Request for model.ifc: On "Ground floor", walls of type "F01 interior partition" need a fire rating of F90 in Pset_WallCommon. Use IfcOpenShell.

First a look at what the model holds.

```python
import ifcopenshell
import ifcopenshell.util.element

model = ifcopenshell.open("model.ifc")
print(model.schema)
storey = next(s for s in model.by_type("IfcBuildingStorey") if s.Name == "Ground floor")
walls = [e for e in ifcopenshell.util.element.get_decomposition(storey) if e.is_a("IfcWall")]
seen = {}
for e in walls:
    element_type = ifcopenshell.util.element.get_type(e)
    key = (element_type.Name if element_type != e and element_type else None, ifcopenshell.util.element.get_pset(e, "Pset_WallCommon", "FireRating"))
    seen[key] = seen.get(key, 0) + 1
for (name, value), count in sorted(seen.items(), key=str):
    print(count, "x", name, "|", value)
```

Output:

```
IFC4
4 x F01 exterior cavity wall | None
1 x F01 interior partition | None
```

```python
import ifcopenshell
import ifcopenshell.api.pset
import ifcopenshell.util.element

model = ifcopenshell.open("model.ifc")

storey = next(s for s in model.by_type("IfcBuildingStorey") if s.Name == "Ground floor")
walls = [e for e in ifcopenshell.util.element.get_decomposition(storey) if e.is_a("IfcWall")]

count = 0
for e in walls:
    element_type = ifcopenshell.util.element.get_type(e)
    if element_type in (None, e) or element_type.Name != "F01 interior partition":
        continue
    # add_pset returns the element's existing set when there is one.
    pset = ifcopenshell.api.pset.add_pset(model, product=e, name="Pset_WallCommon")
    ifcopenshell.api.pset.edit_pset(model, pset=pset, properties={"FireRating": "F90"})
    count += 1

print(count, "walls updated")

model.write("model_updated.ifc")
```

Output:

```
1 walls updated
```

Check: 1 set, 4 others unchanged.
